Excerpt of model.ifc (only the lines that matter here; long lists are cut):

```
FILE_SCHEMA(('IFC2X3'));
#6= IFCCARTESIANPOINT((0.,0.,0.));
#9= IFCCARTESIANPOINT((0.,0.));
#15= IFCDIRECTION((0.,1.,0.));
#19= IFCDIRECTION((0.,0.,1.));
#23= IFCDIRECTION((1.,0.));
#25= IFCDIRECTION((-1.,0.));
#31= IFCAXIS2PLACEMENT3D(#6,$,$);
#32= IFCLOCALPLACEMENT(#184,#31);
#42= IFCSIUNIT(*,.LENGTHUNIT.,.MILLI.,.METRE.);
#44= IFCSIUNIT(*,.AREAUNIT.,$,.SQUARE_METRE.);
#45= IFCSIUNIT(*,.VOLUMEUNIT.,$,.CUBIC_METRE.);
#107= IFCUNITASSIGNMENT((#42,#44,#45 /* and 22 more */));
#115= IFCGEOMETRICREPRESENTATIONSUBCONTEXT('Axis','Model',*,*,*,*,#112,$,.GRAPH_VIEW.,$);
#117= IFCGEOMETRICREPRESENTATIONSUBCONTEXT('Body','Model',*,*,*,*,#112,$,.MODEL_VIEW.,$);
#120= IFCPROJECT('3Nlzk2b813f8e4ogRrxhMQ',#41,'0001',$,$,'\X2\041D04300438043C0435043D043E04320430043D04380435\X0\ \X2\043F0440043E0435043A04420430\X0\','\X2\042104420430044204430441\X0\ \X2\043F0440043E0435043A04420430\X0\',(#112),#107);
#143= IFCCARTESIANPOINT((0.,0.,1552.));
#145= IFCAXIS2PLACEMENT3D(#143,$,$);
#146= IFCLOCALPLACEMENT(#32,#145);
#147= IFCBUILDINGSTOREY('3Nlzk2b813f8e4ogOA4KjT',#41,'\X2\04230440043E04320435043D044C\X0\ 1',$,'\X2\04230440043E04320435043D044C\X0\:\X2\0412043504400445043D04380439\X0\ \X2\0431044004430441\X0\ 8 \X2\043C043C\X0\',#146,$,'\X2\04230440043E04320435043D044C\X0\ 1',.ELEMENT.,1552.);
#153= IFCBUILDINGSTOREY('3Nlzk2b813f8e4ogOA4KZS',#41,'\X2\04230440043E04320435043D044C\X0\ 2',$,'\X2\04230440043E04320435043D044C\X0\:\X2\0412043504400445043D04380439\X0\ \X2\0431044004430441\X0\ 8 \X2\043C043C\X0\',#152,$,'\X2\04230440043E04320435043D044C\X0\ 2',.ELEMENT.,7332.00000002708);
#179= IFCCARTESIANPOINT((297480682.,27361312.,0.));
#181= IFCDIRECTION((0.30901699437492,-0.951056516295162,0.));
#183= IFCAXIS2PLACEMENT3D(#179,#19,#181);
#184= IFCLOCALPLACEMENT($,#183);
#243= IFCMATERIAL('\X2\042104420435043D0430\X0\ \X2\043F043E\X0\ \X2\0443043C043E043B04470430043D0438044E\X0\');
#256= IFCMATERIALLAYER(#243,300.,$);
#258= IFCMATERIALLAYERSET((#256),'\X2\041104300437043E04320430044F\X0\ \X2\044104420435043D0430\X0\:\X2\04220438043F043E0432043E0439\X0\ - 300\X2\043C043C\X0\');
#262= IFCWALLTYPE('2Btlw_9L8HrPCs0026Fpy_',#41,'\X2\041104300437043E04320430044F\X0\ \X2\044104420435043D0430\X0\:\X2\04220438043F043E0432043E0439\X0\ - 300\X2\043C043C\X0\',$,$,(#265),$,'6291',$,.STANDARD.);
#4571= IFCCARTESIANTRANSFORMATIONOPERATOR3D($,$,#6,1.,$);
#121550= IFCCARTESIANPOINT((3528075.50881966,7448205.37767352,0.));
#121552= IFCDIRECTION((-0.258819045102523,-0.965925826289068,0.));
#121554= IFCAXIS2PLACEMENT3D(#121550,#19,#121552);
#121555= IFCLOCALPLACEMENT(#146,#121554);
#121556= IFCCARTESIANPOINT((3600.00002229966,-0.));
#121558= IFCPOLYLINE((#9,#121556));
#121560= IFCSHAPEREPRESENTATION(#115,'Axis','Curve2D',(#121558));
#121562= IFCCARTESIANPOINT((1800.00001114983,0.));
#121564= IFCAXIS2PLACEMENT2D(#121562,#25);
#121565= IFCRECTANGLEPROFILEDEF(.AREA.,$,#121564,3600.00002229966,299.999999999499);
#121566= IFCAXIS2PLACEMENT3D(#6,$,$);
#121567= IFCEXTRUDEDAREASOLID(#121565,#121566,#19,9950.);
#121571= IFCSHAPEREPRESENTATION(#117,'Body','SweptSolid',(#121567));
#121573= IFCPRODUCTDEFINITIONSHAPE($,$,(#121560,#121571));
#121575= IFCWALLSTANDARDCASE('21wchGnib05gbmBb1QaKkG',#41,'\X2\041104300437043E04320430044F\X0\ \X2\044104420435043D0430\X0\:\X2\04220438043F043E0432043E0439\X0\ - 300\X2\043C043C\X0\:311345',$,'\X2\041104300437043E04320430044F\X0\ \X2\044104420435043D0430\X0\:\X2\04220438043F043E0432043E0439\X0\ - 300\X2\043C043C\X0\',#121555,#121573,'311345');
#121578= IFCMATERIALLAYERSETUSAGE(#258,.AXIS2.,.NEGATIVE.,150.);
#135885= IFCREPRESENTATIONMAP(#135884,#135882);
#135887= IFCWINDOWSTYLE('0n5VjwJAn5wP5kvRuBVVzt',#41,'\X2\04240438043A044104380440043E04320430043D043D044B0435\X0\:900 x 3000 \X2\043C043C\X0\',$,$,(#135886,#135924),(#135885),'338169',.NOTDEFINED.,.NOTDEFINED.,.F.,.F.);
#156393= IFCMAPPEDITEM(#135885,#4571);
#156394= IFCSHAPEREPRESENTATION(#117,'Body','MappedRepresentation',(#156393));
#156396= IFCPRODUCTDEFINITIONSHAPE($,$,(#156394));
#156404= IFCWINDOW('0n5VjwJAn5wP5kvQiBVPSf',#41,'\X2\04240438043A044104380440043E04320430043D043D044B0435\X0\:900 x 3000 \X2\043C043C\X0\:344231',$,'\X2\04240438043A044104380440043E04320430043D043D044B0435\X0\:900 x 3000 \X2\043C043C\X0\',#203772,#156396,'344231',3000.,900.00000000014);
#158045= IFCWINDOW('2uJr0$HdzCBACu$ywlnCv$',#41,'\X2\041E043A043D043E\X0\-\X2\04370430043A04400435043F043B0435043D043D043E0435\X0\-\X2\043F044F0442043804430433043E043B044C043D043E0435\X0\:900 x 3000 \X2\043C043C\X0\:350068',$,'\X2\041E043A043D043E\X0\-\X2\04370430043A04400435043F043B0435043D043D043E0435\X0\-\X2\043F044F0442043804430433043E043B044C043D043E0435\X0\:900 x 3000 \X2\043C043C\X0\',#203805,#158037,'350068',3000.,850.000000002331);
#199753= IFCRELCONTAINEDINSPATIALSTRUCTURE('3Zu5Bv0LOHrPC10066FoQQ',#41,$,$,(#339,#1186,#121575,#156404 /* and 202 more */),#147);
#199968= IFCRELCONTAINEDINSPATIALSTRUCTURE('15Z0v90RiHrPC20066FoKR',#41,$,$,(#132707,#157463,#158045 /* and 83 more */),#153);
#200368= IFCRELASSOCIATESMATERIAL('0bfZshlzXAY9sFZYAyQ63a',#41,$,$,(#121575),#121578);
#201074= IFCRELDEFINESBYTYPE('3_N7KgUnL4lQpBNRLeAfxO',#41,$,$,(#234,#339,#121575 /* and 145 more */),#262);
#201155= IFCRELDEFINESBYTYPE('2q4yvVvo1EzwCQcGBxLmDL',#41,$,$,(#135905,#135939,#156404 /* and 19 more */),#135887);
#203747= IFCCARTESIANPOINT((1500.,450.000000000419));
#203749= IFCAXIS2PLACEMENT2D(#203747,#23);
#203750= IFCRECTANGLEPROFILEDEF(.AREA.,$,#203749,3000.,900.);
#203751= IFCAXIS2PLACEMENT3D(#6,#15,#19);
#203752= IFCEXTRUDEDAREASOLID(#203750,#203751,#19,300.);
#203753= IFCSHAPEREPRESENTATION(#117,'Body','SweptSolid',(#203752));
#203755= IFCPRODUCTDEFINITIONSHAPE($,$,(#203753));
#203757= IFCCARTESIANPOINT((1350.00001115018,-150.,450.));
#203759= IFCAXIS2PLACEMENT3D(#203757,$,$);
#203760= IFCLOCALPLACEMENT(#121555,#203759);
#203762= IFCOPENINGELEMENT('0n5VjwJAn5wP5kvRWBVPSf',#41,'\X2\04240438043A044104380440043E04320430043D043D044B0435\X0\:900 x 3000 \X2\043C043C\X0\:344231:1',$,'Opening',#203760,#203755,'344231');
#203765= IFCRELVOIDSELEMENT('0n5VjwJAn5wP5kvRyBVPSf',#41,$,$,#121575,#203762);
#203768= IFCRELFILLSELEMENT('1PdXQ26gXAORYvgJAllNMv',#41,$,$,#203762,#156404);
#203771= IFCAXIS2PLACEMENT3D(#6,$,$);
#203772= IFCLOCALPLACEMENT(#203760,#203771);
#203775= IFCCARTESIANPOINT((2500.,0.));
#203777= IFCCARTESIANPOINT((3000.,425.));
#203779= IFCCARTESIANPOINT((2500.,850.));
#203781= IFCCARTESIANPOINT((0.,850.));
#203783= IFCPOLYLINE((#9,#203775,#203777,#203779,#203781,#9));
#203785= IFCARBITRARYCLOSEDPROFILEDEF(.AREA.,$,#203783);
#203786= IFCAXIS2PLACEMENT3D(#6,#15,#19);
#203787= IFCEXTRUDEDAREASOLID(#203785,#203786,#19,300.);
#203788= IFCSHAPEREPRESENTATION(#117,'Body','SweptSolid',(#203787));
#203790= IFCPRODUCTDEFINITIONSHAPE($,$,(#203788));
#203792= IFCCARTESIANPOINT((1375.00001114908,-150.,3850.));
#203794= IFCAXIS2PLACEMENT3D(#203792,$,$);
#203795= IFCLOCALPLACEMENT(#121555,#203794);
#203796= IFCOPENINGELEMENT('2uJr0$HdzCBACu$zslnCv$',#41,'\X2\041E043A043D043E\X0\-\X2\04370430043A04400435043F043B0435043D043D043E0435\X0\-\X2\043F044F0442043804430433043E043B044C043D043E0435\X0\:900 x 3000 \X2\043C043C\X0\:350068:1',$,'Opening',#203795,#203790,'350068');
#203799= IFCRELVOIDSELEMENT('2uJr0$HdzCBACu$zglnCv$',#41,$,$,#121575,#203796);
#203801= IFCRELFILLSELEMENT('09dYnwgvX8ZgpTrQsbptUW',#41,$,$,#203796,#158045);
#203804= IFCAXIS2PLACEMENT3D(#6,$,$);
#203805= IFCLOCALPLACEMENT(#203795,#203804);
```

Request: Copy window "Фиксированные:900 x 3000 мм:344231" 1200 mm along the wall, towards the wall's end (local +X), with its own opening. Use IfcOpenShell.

```python
import ifcopenshell
import ifcopenshell.api.feature
import ifcopenshell.api.geometry
import ifcopenshell.api.root
import ifcopenshell.geom
import ifcopenshell.util.element
import ifcopenshell.util.placement
import ifcopenshell.util.shape
import ifcopenshell.util.unit

model = ifcopenshell.open("model.ifc")
unit_scale = ifcopenshell.util.unit.calculate_unit_scale(model)
settings = ifcopenshell.geom.settings()


def volume(element):
    """Net volume in cubic metres, openings subtracted."""
    shape = ifcopenshell.geom.create_shape(settings, element)
    return ifcopenshell.util.shape.get_volume(shape.geometry)


def reuse_history(source, copy):
    """copy_class also copies each property set's owner history, people and application; keep the originals."""
    for rel in copy.IsDefinedBy:
        if rel.is_a("IfcRelDefinesByProperties") and (history := rel.RelatingPropertyDefinition.OwnerHistory):
            rel.RelatingPropertyDefinition.OwnerHistory = source.OwnerHistory
            ifcopenshell.util.element.remove_deep2(model, history)


window = model.by_guid("0n5VjwJAn5wP5kvQiBVPSf")
opening = window.FillsVoids[0].RelatingOpeningElement
wall = opening.VoidsElements[0].RelatingBuildingElement
before = volume(wall)
shift = ifcopenshell.util.placement.get_local_placement(wall.ObjectPlacement)[:3, 0] * 1.2 / unit_scale

# copy_class copies the void relationship, type, container and properties, but no geometry.
new_opening = ifcopenshell.api.root.copy_class(model, product=opening)
new_opening.Representation = ifcopenshell.util.element.copy_deep(
    model, opening.Representation, exclude=["IfcGeometricRepresentationContext", "IfcRepresentationMap"]
)
new_opening.Name = "Фиксированные:900 x 3000 мм"
new_opening.Tag = None
new_window = ifcopenshell.api.root.copy_class(model, product=window)
new_window.Representation = ifcopenshell.util.element.copy_deep(
    model, window.Representation, exclude=["IfcGeometricRepresentationContext", "IfcRepresentationMap"]
)
new_window.Name = "Фиксированные:900 x 3000 мм"
new_window.Tag = None
reuse_history(window, new_window)
fills = ifcopenshell.api.feature.add_filling(model, opening=new_opening, element=new_window)
fills.OwnerHistory = new_window.OwnerHistory  # required in IFC2X3

for old, new in ((opening, new_opening), (window, new_window)):
    matrix = ifcopenshell.util.placement.get_local_placement(old.ObjectPlacement)
    matrix[:3, 3] += shift
    ifcopenshell.api.geometry.edit_object_placement(model, product=new, matrix=matrix, is_si=False)

after = volume(wall)

print(f"wall volume {before:.3f} -> {after:.3f} m3")

model.write("model-out.ifc")
```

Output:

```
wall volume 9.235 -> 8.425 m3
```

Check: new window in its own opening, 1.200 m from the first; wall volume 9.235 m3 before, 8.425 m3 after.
